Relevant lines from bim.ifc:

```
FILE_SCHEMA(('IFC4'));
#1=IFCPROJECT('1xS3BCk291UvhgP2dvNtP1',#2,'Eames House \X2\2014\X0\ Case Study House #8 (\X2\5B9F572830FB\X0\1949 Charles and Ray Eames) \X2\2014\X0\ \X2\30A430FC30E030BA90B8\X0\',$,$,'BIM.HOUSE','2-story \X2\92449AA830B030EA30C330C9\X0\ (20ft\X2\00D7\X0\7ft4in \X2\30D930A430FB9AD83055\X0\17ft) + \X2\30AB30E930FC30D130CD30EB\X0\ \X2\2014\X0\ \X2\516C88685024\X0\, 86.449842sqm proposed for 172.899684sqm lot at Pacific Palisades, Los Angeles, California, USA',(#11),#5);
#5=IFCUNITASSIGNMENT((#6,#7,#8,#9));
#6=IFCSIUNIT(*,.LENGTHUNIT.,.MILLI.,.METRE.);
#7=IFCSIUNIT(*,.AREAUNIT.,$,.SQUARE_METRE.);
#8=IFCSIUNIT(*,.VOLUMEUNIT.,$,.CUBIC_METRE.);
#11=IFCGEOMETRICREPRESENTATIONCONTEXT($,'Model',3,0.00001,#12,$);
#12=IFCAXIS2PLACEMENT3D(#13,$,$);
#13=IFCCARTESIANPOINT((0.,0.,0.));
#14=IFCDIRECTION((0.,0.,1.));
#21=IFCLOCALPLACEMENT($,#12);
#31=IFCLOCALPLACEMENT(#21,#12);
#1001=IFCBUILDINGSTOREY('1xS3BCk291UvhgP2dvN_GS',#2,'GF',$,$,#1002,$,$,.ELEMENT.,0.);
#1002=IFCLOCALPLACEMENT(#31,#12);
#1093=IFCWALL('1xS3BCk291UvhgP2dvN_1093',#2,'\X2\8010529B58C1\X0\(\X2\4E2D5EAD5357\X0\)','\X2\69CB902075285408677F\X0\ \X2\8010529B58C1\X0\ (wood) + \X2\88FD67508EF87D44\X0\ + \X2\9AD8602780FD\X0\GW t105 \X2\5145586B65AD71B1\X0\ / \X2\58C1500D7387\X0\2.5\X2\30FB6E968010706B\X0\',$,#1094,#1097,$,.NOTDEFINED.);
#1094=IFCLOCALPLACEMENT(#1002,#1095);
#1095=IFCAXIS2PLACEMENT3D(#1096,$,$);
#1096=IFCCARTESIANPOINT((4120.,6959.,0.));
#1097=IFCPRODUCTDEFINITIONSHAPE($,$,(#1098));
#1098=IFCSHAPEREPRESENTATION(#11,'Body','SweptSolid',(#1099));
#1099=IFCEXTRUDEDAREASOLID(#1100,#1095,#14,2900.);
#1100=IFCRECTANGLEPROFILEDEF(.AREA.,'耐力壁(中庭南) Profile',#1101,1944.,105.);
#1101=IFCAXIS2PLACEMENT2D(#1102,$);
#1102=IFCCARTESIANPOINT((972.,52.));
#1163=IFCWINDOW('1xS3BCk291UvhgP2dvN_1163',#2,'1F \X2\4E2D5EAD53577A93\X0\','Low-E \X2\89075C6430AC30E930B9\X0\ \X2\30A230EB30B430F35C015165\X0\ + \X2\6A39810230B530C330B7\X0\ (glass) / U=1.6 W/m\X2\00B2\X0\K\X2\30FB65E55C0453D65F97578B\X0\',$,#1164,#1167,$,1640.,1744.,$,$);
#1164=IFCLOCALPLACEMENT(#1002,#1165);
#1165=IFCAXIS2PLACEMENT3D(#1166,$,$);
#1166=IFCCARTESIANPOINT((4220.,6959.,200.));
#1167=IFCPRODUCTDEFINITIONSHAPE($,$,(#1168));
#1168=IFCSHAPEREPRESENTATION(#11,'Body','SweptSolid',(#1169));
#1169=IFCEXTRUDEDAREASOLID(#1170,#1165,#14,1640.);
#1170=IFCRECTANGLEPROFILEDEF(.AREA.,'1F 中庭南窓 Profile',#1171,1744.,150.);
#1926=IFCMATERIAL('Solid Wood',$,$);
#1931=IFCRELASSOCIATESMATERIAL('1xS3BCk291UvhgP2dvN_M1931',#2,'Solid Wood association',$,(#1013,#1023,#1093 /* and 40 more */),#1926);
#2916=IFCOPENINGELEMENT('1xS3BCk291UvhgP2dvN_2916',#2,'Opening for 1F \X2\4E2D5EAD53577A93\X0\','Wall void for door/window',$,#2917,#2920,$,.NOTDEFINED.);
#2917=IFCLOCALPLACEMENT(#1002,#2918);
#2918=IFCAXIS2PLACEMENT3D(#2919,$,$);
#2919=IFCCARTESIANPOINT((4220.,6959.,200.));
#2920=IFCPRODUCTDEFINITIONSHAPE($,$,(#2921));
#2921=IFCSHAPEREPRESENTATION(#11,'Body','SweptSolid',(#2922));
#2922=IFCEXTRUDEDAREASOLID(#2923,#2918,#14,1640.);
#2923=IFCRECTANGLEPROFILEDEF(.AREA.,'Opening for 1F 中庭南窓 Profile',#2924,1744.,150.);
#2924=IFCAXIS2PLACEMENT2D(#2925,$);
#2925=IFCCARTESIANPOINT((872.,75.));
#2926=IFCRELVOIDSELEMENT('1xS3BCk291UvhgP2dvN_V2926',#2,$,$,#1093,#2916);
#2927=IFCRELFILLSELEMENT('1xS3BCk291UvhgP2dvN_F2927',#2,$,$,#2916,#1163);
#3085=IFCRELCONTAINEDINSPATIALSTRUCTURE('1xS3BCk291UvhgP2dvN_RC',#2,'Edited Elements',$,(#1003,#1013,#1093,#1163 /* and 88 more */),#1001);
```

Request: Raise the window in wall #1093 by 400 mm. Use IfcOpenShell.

```python
import numpy as np
import ifcopenshell
import ifcopenshell.api.geometry
import ifcopenshell.util.placement
import ifcopenshell.util.unit

model = ifcopenshell.open("bim.ifc")
unit_scale = ifcopenshell.util.unit.calculate_unit_scale(model)

window = model.by_id(1163)
opening = window.FillsVoids[0].RelatingOpeningElement
dz = 0.4 / unit_scale

shift = np.array([0.0, 0.0, dz])
# The window is not placed relative to its opening, so move both.
for product in (opening, window):
    matrix = ifcopenshell.util.placement.get_local_placement(product.ObjectPlacement)
    matrix[:3, 3] += shift
    ifcopenshell.api.geometry.edit_object_placement(model, product=product, matrix=matrix, is_si=False)

print(f"moved by {dz * unit_scale:+.3f} m")

model.write("bim_rev.ifc")
```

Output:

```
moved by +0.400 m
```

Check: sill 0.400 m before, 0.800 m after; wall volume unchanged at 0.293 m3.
